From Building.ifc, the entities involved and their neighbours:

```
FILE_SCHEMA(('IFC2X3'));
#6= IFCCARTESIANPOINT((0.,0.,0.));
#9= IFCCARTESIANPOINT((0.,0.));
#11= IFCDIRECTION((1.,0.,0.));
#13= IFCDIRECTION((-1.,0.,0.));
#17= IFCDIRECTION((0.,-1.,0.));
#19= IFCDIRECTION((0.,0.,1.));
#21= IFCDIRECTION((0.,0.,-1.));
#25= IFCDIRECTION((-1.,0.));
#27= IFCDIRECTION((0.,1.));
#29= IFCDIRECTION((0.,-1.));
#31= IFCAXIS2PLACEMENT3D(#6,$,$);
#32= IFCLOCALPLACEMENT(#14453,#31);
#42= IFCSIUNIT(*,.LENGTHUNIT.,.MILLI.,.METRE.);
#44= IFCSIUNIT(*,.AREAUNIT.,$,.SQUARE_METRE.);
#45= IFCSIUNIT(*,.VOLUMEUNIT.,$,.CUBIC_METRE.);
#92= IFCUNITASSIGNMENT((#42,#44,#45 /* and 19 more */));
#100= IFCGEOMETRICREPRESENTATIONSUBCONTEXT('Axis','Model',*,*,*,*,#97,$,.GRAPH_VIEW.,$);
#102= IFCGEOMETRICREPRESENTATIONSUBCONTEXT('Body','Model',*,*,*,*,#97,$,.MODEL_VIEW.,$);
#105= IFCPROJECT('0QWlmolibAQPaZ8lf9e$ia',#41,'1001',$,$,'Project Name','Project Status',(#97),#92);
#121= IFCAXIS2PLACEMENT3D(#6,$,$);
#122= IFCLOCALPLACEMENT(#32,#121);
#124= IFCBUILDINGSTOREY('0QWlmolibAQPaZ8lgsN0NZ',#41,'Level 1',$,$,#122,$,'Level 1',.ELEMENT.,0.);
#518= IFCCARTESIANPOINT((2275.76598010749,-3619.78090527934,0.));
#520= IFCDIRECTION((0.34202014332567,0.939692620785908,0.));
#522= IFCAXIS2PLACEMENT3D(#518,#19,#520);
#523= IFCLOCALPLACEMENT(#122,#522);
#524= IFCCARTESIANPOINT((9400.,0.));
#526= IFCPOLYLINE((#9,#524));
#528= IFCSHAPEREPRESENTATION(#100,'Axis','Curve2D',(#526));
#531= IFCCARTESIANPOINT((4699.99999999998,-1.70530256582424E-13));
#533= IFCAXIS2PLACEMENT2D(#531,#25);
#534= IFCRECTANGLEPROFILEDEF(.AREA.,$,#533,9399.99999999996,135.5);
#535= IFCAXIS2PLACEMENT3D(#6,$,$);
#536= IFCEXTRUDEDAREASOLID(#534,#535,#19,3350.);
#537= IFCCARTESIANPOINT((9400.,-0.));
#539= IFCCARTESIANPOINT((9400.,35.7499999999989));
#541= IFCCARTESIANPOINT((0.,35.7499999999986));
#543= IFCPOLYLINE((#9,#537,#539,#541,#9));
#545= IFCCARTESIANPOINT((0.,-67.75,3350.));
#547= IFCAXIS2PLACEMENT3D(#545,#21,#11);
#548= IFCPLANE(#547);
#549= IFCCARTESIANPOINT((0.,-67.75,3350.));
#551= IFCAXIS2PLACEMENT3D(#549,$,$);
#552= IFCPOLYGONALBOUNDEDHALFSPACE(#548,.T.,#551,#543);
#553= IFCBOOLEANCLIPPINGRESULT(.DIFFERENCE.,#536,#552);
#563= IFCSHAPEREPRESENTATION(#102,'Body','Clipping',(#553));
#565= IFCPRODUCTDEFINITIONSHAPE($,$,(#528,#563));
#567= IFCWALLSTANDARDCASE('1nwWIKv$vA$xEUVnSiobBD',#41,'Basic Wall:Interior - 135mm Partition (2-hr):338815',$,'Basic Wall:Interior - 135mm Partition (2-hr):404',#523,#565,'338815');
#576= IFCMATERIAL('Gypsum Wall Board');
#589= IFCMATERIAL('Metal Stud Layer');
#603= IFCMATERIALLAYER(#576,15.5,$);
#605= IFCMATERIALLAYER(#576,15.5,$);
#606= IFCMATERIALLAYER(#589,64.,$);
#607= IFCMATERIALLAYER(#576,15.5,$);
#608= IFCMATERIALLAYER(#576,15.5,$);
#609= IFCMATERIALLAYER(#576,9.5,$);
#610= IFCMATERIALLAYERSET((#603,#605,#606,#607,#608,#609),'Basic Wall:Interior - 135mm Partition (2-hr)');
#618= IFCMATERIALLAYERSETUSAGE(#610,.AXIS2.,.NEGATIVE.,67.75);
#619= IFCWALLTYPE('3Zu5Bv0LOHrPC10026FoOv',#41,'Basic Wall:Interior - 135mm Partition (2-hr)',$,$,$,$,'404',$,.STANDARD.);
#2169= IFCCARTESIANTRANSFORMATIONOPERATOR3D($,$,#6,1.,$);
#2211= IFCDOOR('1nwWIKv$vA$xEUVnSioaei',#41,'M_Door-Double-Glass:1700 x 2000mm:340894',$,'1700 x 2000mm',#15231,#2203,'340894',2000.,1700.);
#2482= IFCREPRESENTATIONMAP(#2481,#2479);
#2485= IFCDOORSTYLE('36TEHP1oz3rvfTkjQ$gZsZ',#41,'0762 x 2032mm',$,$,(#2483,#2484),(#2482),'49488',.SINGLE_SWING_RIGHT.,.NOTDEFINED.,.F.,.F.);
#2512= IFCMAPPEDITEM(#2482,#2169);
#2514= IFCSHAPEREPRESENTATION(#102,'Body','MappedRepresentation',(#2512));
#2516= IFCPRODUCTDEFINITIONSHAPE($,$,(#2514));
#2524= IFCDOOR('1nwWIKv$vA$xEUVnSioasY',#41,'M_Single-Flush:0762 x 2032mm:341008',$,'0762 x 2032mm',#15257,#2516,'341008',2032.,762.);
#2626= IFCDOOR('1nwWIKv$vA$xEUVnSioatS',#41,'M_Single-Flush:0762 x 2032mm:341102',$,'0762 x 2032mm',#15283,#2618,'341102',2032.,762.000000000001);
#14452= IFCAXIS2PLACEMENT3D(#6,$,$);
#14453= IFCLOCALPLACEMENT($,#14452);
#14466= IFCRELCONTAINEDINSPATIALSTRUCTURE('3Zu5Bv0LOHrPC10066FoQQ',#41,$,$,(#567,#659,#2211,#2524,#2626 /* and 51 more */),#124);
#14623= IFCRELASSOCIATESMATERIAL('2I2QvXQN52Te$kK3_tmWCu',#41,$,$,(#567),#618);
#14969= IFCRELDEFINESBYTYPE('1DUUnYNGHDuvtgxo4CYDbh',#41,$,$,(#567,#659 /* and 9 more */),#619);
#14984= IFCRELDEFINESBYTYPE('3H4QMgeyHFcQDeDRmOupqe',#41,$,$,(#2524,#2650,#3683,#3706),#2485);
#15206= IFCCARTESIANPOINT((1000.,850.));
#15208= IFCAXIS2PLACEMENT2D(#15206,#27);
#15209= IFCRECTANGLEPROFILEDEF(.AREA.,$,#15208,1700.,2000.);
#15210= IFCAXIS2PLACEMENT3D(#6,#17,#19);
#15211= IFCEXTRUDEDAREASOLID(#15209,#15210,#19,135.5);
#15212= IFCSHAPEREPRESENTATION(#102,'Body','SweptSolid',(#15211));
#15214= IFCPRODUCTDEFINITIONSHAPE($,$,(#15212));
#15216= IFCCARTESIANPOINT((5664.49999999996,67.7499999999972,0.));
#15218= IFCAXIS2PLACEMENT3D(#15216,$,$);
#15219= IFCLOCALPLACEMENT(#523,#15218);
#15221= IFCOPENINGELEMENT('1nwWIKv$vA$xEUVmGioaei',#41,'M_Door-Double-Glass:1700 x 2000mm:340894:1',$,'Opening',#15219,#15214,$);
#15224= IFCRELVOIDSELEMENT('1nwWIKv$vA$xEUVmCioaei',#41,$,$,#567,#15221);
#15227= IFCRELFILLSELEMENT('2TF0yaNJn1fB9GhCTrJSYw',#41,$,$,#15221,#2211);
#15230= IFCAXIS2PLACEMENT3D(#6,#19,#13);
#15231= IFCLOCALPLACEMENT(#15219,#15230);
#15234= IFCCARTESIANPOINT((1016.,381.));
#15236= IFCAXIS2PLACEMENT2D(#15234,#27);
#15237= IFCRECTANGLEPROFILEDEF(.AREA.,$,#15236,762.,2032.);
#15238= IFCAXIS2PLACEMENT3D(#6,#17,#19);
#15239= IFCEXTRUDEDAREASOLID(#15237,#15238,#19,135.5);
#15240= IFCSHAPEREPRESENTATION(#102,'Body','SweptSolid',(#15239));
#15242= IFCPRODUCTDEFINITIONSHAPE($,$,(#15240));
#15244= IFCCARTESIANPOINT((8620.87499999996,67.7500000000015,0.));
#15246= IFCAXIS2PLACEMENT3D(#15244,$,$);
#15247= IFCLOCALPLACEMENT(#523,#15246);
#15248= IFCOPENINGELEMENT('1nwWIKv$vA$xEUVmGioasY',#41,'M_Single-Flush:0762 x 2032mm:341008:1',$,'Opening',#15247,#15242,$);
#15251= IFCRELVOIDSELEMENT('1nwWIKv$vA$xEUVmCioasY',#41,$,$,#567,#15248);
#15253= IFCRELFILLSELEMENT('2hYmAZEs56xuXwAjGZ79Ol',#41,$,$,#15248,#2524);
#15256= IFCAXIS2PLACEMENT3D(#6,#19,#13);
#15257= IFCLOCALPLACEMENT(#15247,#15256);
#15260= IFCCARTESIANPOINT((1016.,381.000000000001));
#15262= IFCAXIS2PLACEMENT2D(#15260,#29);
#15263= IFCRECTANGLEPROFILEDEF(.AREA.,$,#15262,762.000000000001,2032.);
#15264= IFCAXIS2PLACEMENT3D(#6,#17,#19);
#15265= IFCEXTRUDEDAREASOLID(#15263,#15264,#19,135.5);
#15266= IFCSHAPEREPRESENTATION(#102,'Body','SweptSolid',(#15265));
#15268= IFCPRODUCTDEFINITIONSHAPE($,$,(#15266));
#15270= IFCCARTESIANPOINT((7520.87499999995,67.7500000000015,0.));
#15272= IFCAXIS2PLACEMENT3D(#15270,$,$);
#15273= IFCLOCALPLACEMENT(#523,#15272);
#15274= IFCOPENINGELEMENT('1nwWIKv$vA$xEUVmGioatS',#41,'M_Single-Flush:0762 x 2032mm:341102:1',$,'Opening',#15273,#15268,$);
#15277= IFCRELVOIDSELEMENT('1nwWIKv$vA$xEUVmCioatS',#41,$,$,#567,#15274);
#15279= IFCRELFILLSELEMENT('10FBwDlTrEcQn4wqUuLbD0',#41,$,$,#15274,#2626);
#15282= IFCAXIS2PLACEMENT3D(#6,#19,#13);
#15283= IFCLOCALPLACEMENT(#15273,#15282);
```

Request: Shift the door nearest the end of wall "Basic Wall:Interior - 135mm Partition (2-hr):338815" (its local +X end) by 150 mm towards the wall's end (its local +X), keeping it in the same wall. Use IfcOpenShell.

```python
import ifcopenshell
import ifcopenshell.api.geometry
import ifcopenshell.util.placement

model = ifcopenshell.open("Building.ifc")

door = model.by_guid("1nwWIKv$vA$xEUVnSioasY")
opening = door.FillsVoids[0].RelatingOpeningElement
wall = opening.VoidsElements[0].RelatingBuildingElement

wall_matrix = ifcopenshell.util.placement.get_local_placement(wall.ObjectPlacement)
shift = wall_matrix[:3, 0] * 150.0
before = ifcopenshell.util.placement.get_local_placement(door.ObjectPlacement)[:3, 3].copy()

# The door is placed relative to its opening, so it follows when the opening moves.
matrix = ifcopenshell.util.placement.get_local_placement(opening.ObjectPlacement)
matrix[:3, 3] += shift
ifcopenshell.api.geometry.edit_object_placement(
    model, product=opening, matrix=matrix, is_si=False, should_transform_children=True
)

after = ifcopenshell.util.placement.get_local_placement(door.ObjectPlacement)[:3, 3]
print("door moved by", (after - before).round(3) + 0.0)

model.write("Building_rev.ifc")
```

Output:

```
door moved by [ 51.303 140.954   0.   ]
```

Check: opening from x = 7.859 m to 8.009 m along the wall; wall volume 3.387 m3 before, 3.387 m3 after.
